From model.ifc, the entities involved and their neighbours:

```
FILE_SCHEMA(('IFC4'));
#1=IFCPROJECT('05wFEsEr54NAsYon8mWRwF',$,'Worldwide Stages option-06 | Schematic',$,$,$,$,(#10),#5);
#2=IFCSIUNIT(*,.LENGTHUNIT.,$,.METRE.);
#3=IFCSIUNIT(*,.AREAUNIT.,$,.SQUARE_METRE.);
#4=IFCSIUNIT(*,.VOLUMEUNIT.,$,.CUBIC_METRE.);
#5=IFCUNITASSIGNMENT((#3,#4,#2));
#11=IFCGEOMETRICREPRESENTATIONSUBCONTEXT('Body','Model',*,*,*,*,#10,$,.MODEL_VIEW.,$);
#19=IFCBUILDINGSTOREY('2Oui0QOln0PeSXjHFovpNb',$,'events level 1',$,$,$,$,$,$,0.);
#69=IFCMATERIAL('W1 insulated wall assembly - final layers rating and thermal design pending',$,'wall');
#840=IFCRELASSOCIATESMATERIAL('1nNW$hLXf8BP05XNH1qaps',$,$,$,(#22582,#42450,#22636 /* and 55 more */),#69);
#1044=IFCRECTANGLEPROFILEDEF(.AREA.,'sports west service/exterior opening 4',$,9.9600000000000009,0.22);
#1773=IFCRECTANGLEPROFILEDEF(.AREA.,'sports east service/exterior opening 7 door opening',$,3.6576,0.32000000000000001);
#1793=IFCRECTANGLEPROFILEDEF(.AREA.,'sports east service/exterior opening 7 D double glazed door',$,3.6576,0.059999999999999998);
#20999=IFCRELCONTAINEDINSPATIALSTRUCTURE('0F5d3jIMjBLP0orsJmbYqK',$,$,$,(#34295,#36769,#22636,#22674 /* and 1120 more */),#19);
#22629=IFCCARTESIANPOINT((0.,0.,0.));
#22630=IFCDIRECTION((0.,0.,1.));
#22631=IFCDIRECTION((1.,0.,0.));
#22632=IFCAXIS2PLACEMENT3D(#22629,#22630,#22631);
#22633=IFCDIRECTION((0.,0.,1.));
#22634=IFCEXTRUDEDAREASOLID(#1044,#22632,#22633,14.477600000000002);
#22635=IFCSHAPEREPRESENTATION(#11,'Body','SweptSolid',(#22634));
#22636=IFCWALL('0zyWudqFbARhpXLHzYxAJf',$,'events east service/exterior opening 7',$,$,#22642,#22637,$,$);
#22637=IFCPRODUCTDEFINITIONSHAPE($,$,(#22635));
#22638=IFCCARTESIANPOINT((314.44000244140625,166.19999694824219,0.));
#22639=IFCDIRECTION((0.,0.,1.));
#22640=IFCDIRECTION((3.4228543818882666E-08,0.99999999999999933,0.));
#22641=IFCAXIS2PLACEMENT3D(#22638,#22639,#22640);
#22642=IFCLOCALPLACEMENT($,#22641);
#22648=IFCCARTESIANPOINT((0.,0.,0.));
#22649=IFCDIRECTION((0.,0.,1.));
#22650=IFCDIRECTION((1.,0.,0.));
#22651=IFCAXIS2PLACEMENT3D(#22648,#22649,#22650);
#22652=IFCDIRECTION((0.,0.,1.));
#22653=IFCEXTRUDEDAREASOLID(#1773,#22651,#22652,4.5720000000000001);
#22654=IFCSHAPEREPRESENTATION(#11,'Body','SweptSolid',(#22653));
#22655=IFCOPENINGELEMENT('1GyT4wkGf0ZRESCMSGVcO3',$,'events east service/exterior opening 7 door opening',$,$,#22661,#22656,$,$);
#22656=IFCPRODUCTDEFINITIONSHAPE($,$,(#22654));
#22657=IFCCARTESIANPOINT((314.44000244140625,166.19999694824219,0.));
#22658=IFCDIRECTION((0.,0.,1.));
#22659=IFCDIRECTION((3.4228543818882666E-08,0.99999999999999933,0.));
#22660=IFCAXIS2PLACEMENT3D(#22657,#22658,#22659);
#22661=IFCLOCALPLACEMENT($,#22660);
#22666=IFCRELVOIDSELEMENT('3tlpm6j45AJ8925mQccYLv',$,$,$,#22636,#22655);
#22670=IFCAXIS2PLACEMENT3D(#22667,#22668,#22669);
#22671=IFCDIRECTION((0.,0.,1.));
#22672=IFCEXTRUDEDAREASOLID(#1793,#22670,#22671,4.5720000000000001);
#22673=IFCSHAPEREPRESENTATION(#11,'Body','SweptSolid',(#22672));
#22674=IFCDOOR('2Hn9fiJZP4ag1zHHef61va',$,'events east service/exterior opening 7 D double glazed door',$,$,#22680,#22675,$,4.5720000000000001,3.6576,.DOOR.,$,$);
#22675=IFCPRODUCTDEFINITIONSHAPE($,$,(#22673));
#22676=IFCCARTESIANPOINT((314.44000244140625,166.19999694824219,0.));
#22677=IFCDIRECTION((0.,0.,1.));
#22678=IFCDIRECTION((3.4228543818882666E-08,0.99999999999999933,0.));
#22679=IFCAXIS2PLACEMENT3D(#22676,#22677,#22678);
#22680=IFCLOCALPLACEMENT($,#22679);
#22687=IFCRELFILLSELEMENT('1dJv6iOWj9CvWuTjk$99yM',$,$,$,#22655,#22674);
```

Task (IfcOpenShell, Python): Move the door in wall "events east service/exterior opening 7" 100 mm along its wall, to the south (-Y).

```python
import ifcopenshell
import ifcopenshell.api.geometry
import ifcopenshell.util.placement
import ifcopenshell.util.unit

model = ifcopenshell.open("model.ifc")
unit_scale = ifcopenshell.util.unit.calculate_unit_scale(model)

door = model.by_guid("2Hn9fiJZP4ag1zHHef61va")
opening = door.FillsVoids[0].RelatingOpeningElement
wall = opening.VoidsElements[0].RelatingBuildingElement

wall_matrix = ifcopenshell.util.placement.get_local_placement(wall.ObjectPlacement)
shift = wall_matrix[:3, 0] * -0.1 / unit_scale
before = ifcopenshell.util.placement.get_local_placement(door.ObjectPlacement)[:3, 3].copy()

# The door is not placed relative to its opening, so move both.
for product in (opening, door):
    matrix = ifcopenshell.util.placement.get_local_placement(product.ObjectPlacement)
    matrix[:3, 3] += shift
    ifcopenshell.api.geometry.edit_object_placement(model, product=product, matrix=matrix, is_si=False)

after = ifcopenshell.util.placement.get_local_placement(door.ObjectPlacement)[:3, 3]
print("door moved by", (after - before).round(3) + 0.0)

model.write("model_v2.ifc")
```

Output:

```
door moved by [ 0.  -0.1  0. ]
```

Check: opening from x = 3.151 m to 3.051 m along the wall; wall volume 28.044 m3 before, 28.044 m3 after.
